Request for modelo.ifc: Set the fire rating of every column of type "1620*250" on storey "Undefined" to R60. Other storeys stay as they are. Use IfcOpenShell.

First a look at what the model holds.

```python
import ifcopenshell
import ifcopenshell.util.element

model = ifcopenshell.open("modelo.ifc")
print(model.schema)
storey = next(s for s in model.by_type("IfcBuildingStorey") if s.Name == "Undefined")
columns = [e for e in ifcopenshell.util.element.get_decomposition(storey) if e.is_a("IfcColumn")]
seen = {}
for e in columns:
    element_type = ifcopenshell.util.element.get_type(e)
    key = (element_type.Name if element_type != e and element_type else None, ifcopenshell.util.element.get_pset(e, "Pset_ColumnCommon", "FireRating"))
    seen[key] = seen.get(key, 0) + 1
for (name, value), count in sorted(seen.items(), key=str):
    print(count, "x", name, "|", value)
```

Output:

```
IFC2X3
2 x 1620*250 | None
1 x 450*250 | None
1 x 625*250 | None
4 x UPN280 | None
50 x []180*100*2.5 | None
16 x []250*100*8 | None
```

```python
import ifcopenshell
import ifcopenshell.api.pset
import ifcopenshell.util.element

model = ifcopenshell.open("modelo.ifc")

storey = next(s for s in model.by_type("IfcBuildingStorey") if s.Name == "Undefined")
columns = [e for e in ifcopenshell.util.element.get_decomposition(storey) if e.is_a("IfcColumn")]

count = 0
for e in columns:
    element_type = ifcopenshell.util.element.get_type(e)
    if element_type in (None, e) or element_type.Name != "1620*250":
        continue
    found = ifcopenshell.util.element.get_pset(e, "Pset_ColumnCommon", should_inherit=False)
    if found:
        pset = model.by_id(found["id"])
        if len(ifcopenshell.util.element.get_elements_by_pset(pset)) > 1:
            pset = ifcopenshell.api.pset.unshare_pset(model, products=[e], pset=pset)[0]
    else:
        pset = ifcopenshell.api.pset.add_pset(model, product=e, name="Pset_ColumnCommon")
    ifcopenshell.api.pset.edit_pset(model, pset=pset, properties={"FireRating": "R60"})
    count += 1

print(count, "columns updated")

model.write("modelo_v2.ifc")
```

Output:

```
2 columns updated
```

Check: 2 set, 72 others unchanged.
